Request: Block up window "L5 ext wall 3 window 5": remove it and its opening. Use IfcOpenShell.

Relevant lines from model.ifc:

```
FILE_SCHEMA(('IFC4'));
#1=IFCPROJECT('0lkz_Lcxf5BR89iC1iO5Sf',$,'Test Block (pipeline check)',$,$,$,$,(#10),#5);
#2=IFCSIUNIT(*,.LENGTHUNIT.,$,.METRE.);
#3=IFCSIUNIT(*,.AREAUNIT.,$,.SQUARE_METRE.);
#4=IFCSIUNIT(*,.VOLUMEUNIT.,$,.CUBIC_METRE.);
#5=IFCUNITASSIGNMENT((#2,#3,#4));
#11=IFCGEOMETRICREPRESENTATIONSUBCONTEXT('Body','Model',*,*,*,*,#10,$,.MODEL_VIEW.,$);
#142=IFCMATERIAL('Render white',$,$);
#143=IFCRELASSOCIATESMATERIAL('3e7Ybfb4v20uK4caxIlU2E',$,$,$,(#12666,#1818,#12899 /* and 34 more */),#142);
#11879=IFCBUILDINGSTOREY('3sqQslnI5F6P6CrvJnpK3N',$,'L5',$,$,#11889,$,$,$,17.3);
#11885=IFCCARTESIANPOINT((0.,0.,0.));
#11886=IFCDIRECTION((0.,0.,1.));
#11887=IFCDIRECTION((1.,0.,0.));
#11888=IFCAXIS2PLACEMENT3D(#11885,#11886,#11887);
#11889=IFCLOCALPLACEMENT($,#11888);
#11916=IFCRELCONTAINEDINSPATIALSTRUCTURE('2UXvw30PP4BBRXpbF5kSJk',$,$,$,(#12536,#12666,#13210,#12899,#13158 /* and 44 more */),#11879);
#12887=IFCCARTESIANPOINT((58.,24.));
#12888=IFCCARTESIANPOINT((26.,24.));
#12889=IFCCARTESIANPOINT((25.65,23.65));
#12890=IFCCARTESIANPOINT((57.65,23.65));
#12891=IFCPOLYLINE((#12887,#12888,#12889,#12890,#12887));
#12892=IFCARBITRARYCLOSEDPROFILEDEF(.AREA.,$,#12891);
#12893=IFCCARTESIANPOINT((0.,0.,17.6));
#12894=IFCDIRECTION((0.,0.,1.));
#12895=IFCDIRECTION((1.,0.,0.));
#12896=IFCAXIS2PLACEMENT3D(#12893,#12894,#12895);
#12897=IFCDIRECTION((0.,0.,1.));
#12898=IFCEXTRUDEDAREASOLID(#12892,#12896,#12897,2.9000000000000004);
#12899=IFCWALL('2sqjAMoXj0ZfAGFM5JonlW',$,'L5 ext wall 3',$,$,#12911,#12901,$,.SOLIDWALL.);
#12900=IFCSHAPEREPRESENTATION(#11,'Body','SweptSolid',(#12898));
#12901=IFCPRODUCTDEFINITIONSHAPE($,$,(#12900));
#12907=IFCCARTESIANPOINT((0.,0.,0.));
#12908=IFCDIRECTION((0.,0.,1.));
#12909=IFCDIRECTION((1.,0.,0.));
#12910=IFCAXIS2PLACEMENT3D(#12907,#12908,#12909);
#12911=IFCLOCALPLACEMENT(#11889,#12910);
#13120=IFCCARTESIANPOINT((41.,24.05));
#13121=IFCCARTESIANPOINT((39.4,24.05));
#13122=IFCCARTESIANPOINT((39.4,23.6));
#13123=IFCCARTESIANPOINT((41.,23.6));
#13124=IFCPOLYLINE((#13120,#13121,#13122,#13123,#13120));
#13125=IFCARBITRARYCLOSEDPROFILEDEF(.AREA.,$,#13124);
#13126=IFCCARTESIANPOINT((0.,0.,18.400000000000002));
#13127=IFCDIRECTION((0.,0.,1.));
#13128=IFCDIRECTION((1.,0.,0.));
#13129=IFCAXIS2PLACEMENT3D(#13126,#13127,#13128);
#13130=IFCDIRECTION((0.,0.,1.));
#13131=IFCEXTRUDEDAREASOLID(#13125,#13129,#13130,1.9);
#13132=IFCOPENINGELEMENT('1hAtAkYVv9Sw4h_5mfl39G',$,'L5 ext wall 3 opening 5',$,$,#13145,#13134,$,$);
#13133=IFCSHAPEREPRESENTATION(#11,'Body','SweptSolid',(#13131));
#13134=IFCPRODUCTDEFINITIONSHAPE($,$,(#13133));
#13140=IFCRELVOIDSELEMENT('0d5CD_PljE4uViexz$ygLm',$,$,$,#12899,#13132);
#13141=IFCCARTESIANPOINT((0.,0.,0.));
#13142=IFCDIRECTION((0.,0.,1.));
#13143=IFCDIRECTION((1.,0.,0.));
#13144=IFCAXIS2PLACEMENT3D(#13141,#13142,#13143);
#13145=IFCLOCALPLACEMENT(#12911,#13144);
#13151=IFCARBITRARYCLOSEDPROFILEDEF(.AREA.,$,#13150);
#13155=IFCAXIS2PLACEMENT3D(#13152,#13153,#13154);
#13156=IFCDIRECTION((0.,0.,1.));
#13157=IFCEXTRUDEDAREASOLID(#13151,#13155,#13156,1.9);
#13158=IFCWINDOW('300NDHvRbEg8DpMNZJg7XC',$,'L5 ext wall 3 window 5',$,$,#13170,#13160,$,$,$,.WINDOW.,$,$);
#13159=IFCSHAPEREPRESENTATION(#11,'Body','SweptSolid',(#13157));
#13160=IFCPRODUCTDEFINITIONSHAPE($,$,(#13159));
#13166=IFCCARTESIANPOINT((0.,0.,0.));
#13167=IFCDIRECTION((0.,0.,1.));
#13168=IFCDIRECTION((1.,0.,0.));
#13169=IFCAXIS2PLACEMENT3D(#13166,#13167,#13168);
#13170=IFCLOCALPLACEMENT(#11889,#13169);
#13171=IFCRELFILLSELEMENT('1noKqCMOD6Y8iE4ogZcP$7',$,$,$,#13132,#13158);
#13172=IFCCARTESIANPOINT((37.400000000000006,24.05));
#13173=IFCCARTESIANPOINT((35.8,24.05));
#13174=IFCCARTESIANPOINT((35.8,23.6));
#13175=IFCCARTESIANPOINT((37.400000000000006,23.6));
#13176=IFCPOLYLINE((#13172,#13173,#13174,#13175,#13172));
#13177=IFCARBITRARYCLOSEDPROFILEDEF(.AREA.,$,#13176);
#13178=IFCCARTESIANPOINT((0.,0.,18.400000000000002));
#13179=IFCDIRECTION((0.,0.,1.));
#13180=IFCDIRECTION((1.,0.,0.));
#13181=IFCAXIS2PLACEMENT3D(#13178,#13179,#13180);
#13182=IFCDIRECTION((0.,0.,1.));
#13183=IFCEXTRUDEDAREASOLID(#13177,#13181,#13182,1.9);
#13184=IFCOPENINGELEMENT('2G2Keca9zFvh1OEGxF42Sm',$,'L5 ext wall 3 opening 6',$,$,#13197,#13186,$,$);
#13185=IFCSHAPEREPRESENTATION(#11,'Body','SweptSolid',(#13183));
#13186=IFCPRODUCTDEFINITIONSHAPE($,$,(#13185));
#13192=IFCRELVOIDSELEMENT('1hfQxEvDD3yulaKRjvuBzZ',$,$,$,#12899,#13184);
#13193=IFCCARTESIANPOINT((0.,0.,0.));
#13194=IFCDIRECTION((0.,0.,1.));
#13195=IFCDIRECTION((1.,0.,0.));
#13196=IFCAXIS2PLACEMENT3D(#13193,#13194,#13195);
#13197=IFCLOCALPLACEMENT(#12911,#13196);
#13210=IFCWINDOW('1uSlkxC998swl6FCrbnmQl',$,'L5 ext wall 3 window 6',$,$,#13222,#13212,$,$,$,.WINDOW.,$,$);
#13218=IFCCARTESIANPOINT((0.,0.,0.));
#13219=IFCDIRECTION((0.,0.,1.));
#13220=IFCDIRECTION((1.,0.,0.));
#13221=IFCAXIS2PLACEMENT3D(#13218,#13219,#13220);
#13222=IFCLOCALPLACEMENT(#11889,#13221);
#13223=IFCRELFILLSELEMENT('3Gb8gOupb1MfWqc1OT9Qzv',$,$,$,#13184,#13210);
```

```python
import ifcopenshell
import ifcopenshell.api.feature
import ifcopenshell.api.root
import ifcopenshell.geom
import ifcopenshell.util.shape

model = ifcopenshell.open("model.ifc")
settings = ifcopenshell.geom.settings()


def volume(element):
    """Net volume in cubic metres, openings subtracted."""
    shape = ifcopenshell.geom.create_shape(settings, element)
    return ifcopenshell.util.shape.get_volume(shape.geometry)


window = model.by_guid("300NDHvRbEg8DpMNZJg7XC")
opening = window.FillsVoids[0].RelatingOpeningElement
wall = opening.VoidsElements[0].RelatingBuildingElement
before = volume(wall)

ifcopenshell.api.root.remove_product(model, product=window)
ifcopenshell.api.feature.remove_feature(model, feature=opening)

after = volume(wall)

print(f"wall volume {before:.3f} -> {after:.3f} m3")

model.write("model_edited.ifc")
```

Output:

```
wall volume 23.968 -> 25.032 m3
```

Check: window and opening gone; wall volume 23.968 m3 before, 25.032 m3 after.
